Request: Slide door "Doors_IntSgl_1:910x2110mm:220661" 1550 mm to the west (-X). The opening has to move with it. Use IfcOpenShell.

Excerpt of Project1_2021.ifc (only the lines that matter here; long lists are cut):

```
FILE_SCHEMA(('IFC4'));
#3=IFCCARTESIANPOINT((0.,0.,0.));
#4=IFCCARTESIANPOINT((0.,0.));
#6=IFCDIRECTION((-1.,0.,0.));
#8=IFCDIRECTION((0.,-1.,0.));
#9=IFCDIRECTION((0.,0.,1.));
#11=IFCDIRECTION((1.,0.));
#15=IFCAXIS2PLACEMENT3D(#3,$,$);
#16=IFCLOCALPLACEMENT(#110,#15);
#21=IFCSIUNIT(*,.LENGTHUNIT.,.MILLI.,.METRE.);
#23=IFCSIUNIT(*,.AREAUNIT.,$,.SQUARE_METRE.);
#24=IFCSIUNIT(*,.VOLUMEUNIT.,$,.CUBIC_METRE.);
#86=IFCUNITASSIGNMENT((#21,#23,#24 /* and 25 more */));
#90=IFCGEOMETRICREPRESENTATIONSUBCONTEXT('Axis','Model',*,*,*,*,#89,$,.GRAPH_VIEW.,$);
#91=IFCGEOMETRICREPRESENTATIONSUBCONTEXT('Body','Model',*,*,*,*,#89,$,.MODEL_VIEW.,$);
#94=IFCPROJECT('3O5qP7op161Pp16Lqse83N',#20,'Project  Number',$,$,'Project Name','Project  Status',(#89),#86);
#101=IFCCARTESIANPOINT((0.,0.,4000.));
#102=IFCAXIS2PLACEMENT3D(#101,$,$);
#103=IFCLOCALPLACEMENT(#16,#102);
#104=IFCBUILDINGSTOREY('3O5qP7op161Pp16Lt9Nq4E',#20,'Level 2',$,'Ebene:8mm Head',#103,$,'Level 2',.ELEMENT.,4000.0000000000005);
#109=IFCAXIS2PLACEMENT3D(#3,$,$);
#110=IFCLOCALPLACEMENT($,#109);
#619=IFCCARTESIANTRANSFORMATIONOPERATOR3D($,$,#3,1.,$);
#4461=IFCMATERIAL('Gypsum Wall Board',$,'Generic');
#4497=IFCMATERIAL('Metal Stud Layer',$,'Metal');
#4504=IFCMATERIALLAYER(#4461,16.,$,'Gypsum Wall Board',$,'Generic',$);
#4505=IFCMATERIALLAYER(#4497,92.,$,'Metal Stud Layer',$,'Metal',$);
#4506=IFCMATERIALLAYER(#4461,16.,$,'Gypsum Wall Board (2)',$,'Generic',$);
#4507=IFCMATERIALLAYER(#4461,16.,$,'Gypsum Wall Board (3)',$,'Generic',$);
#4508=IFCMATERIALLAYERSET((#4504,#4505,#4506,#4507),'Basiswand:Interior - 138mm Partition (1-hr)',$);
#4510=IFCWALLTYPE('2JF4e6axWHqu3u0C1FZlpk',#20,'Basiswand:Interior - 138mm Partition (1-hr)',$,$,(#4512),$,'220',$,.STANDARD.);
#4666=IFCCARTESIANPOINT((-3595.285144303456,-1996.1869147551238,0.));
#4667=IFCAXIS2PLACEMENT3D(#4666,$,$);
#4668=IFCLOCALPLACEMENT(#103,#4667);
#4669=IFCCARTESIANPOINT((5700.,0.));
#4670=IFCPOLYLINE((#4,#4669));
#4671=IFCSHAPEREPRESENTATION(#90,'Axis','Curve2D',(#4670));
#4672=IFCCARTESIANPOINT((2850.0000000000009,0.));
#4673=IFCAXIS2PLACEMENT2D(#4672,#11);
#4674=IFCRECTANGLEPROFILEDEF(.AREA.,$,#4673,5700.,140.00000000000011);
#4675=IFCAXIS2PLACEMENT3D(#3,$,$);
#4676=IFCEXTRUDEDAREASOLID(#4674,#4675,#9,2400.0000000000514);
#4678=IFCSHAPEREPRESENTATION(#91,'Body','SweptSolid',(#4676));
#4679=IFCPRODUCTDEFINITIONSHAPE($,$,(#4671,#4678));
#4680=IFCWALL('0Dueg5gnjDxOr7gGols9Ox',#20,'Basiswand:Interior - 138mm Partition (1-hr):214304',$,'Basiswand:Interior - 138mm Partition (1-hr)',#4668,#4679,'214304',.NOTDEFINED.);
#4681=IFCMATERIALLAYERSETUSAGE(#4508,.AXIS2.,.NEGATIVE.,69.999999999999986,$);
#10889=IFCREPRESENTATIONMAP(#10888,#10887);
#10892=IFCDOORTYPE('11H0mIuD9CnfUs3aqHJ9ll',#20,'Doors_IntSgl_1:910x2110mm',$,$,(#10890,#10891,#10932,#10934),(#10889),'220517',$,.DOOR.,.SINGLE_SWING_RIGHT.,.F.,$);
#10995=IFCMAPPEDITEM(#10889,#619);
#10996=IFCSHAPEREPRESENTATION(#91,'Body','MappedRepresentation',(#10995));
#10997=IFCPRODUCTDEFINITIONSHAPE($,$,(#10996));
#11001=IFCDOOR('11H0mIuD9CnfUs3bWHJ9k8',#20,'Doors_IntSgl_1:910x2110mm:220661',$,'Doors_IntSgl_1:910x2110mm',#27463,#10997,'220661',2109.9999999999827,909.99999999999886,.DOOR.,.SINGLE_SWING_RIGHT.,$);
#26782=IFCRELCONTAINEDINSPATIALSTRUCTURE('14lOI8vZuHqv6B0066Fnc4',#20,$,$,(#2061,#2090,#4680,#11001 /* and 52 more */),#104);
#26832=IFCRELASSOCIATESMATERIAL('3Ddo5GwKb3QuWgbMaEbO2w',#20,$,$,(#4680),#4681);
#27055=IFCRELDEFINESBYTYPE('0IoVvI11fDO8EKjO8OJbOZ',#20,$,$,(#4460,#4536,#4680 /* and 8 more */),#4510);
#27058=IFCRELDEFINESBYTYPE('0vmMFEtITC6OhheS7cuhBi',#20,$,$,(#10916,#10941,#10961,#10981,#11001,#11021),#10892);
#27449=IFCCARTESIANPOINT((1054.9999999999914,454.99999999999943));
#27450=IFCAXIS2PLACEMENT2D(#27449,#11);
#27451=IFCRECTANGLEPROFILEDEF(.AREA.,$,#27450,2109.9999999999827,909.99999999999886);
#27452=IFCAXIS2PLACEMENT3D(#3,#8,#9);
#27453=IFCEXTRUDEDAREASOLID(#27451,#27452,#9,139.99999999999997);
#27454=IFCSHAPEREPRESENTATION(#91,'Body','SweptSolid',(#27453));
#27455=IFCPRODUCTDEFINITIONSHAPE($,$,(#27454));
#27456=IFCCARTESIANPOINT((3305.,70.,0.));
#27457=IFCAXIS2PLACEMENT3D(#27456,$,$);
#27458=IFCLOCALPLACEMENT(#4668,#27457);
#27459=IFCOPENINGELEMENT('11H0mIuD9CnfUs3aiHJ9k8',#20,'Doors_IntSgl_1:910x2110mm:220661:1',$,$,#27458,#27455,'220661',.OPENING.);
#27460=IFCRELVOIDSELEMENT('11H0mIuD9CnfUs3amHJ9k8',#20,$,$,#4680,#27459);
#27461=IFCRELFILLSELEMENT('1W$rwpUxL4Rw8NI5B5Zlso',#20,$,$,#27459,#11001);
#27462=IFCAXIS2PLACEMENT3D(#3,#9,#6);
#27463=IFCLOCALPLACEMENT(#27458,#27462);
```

```python
import ifcopenshell
import ifcopenshell.api.geometry
import ifcopenshell.util.placement

model = ifcopenshell.open("Project1_2021.ifc")

door = model.by_id(11001)
opening = door.FillsVoids[0].RelatingOpeningElement
wall = opening.VoidsElements[0].RelatingBuildingElement

wall_matrix = ifcopenshell.util.placement.get_local_placement(wall.ObjectPlacement)
shift = wall_matrix[:3, 0] * -1550.0
before = ifcopenshell.util.placement.get_local_placement(door.ObjectPlacement)[:3, 3].copy()

# The door is placed relative to its opening, so it follows when the opening moves.
matrix = ifcopenshell.util.placement.get_local_placement(opening.ObjectPlacement)
matrix[:3, 3] += shift
ifcopenshell.api.geometry.edit_object_placement(
    model, product=opening, matrix=matrix, is_si=False, should_transform_children=True
)

after = ifcopenshell.util.placement.get_local_placement(door.ObjectPlacement)[:3, 3]
print("door moved by", (after - before).round(3) + 0.0)

model.write("Project1_2021_rev.ifc")
```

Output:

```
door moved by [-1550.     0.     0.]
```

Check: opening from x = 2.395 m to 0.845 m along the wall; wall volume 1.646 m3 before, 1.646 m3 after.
